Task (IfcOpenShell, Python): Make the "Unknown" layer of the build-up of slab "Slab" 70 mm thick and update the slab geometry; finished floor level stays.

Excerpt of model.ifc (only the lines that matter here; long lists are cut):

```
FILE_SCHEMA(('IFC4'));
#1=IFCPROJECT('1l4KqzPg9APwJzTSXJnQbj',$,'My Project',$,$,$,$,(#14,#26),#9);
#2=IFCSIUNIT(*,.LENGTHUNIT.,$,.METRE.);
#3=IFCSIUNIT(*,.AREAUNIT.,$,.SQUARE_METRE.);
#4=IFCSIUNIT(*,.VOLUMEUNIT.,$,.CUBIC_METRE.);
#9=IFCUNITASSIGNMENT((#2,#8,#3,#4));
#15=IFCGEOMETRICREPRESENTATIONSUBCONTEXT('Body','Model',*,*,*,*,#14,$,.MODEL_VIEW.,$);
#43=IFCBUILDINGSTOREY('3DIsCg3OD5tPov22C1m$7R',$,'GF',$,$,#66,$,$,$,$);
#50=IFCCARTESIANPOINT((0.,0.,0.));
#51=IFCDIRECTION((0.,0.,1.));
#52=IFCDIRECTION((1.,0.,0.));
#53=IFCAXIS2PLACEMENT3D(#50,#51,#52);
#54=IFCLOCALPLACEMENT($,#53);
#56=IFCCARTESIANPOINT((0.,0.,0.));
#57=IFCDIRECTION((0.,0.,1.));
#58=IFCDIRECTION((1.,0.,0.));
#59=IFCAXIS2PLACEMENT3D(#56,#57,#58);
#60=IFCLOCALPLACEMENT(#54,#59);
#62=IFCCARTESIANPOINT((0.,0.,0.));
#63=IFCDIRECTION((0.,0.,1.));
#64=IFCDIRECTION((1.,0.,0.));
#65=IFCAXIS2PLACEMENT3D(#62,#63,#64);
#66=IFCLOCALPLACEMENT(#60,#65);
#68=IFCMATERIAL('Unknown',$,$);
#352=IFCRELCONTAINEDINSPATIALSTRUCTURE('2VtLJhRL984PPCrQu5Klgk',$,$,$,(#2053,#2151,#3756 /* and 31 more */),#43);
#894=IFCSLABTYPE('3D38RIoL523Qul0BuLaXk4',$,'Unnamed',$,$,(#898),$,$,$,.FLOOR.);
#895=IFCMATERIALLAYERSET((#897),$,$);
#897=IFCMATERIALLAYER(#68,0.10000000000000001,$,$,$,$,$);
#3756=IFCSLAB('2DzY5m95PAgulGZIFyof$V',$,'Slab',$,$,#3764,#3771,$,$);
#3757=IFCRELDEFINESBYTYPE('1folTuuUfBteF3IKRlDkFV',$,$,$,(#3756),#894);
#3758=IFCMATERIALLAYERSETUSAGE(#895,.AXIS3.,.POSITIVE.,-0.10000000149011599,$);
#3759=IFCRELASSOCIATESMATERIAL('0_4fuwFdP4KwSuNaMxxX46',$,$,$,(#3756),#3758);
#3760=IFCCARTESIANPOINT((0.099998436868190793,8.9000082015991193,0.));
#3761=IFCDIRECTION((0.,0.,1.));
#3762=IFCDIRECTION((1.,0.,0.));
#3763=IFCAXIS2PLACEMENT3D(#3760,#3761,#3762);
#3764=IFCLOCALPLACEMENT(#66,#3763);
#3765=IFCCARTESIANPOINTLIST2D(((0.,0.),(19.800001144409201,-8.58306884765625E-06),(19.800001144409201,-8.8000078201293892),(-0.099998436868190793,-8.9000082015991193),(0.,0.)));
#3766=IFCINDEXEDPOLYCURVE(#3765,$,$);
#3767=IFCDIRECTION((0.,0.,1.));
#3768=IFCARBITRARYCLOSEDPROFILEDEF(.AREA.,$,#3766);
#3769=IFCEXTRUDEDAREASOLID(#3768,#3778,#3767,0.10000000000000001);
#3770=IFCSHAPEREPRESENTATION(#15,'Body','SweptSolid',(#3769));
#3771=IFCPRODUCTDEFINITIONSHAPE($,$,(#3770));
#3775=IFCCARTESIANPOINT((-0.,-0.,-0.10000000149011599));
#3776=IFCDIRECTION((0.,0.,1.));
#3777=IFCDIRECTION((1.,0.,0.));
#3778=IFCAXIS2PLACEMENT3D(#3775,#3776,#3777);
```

```python
import ifcopenshell
import ifcopenshell.util.element
import ifcopenshell.util.representation
import ifcopenshell.util.unit

model = ifcopenshell.open("model.ifc")
unit_scale = ifcopenshell.util.unit.calculate_unit_scale(model)

layer_set = model.by_id(895)
layer = next(l for l in layer_set.MaterialLayers if l.Material and l.Material.Name == "Unknown")
change = 0.07 / unit_scale - layer.LayerThickness
layer.LayerThickness += change

# Geometry does not follow the layer set by itself.
slabs = [e for e in ifcopenshell.util.element.get_elements_by_material(model, layer_set) if e.is_a("IfcSlab")]
for slab in sorted(slabs, key=lambda e: e.id()):
    body = ifcopenshell.util.representation.get_representation(slab, "Model", "Body")
    solid = body.Items[0]
    old_depth = solid.Depth
    solid.Depth += change
    # Extruded upwards: lower the start of the extrusion so the top stays.
    x, y, z = solid.Position.Location.Coordinates
    solid.Position.Location = model.createIfcCartesianPoint((x, y, z - change))
    print(slab.id(), f"{old_depth:g} -> {solid.Depth:g}")

# The layers are counted up from the underside, which has moved.
for usage in {ifcopenshell.util.element.get_material(slab) for slab in slabs}:
    usage.OffsetFromReferenceLine -= change

model.write("model_v2.ifc")
```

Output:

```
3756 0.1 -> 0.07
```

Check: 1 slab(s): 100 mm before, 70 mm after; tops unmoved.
